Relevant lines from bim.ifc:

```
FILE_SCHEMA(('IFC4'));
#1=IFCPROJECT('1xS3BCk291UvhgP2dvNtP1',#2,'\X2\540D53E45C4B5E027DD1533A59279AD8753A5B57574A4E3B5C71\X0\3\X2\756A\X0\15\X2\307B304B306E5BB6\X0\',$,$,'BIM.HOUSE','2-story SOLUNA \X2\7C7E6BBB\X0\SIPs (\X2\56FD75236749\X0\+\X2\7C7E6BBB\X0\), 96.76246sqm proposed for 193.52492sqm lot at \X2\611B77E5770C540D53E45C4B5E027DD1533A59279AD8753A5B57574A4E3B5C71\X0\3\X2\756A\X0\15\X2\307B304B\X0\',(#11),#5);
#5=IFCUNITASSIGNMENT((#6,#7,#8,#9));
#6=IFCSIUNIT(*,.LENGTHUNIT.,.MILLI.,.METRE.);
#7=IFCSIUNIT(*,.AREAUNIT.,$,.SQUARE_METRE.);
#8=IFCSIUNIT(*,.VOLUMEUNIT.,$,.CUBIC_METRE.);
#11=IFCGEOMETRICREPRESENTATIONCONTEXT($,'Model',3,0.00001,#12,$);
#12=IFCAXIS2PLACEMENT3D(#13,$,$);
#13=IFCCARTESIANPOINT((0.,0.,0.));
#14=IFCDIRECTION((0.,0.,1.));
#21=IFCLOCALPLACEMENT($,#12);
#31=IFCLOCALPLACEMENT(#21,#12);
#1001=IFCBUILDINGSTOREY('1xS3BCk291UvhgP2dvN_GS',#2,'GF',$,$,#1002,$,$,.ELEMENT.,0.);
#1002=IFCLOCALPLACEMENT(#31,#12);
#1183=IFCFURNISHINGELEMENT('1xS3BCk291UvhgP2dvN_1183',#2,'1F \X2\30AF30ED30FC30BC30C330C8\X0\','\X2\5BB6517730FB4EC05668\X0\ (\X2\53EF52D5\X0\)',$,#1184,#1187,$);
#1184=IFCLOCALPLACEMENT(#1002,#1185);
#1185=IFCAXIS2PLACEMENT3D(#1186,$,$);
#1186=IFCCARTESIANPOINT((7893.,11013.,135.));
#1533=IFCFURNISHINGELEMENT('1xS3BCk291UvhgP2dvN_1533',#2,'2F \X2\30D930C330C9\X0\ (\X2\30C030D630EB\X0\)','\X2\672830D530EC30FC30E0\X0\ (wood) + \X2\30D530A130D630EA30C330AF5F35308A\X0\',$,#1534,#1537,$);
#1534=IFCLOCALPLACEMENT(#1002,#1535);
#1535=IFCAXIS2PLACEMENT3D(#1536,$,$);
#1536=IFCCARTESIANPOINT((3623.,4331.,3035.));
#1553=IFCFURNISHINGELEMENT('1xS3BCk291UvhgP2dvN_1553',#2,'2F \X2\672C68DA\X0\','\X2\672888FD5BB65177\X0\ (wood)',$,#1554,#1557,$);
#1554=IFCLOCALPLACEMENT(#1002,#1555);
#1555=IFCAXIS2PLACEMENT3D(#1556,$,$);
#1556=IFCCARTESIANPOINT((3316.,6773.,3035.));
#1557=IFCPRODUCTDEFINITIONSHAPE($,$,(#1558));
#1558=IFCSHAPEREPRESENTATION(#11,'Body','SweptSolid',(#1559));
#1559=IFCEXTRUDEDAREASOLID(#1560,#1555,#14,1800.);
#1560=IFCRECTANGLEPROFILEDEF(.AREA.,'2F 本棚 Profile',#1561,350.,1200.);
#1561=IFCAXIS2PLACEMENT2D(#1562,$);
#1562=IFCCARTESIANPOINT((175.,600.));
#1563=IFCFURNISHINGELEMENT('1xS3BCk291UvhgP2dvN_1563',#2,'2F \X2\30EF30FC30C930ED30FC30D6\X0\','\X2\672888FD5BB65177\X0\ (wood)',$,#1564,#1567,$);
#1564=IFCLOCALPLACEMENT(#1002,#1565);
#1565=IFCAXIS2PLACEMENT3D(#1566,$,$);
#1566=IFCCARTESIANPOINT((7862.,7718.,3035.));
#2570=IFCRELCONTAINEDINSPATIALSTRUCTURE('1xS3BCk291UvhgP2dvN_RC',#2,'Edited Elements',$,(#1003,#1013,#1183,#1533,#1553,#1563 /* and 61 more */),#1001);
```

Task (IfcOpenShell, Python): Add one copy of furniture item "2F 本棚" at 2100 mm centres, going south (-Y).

```python
import numpy as np
import ifcopenshell
import ifcopenshell.api.geometry
import ifcopenshell.api.root
import ifcopenshell.util.element
import ifcopenshell.util.placement

model = ifcopenshell.open("bim.ifc")


def reuse_history(source, copy):
    """copy_class also copies each property set's owner history, people and application; keep the originals."""
    for rel in copy.IsDefinedBy:
        if rel.is_a("IfcRelDefinesByProperties") and (history := rel.RelatingPropertyDefinition.OwnerHistory):
            rel.RelatingPropertyDefinition.OwnerHistory = source.OwnerHistory
            ifcopenshell.util.element.remove_deep2(model, history)


source = model.by_guid("1xS3BCk291UvhgP2dvN_1553")
base = ifcopenshell.util.placement.get_local_placement(source.ObjectPlacement)
step = np.array([0.0, -1.0, 0.0]) * 2100.0

for i in range(1, 2):
    copy = ifcopenshell.api.root.copy_class(model, product=source)
    copy.Representation = ifcopenshell.util.element.copy_deep(
        model, source.Representation, exclude=["IfcGeometricRepresentationContext", "IfcRepresentationMap"]
    )
    reuse_history(source, copy)
    matrix = base.copy()
    matrix[:3, 3] += i * step
    print("added at", matrix[:3, 3].round(3) + 0.0)
    ifcopenshell.api.geometry.edit_object_placement(model, product=copy, matrix=matrix, is_si=False)

model.write("bim_v2.ifc")
```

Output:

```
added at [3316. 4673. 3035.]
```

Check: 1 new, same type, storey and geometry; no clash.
